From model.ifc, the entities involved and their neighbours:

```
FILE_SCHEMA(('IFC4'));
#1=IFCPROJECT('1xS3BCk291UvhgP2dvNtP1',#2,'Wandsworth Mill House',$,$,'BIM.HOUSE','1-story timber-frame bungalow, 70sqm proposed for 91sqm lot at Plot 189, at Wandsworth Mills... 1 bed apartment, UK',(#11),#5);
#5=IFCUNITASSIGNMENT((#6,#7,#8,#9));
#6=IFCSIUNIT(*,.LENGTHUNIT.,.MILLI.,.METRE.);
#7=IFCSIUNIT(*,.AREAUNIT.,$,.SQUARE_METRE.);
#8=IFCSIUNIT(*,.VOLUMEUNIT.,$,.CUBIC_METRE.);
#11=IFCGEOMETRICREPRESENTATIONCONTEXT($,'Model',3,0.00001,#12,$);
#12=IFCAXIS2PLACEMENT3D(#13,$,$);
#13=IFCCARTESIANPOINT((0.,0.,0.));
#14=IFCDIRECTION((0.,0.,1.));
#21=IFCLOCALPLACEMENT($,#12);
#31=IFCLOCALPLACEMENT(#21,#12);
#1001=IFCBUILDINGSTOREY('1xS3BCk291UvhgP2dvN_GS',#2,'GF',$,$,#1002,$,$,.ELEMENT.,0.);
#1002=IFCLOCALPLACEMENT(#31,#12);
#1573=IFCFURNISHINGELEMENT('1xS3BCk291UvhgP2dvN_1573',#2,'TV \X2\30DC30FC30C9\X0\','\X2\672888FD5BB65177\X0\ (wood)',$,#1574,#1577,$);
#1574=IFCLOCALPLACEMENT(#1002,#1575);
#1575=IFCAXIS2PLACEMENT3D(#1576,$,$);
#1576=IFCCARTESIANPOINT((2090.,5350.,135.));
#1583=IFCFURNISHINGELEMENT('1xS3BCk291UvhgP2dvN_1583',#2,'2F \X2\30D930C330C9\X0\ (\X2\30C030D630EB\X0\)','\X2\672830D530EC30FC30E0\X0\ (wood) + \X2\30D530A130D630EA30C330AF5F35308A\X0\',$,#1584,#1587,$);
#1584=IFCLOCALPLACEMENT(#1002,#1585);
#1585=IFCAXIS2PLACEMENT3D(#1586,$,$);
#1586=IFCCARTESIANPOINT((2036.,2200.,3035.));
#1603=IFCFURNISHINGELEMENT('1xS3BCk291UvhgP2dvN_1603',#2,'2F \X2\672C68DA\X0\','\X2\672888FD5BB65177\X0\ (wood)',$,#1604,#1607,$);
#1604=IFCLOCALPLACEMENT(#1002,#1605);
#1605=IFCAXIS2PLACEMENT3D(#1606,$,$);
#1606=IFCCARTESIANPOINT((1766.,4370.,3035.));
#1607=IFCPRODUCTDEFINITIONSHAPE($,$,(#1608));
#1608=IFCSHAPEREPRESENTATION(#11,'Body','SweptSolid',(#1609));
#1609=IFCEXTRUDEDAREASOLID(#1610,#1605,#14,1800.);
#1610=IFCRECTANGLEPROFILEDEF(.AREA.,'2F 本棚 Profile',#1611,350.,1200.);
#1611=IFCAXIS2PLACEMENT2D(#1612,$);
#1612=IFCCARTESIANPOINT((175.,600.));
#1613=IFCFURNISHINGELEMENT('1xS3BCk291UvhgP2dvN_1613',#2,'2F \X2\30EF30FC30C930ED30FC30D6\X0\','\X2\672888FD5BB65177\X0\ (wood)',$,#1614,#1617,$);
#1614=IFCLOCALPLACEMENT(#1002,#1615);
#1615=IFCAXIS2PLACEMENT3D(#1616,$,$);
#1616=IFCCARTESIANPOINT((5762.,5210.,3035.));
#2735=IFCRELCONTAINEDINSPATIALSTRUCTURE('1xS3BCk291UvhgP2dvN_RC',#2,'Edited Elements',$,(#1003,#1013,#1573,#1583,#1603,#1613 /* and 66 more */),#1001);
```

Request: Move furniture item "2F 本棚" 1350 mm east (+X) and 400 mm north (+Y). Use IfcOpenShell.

```python
import ifcopenshell
import ifcopenshell.api.geometry
import ifcopenshell.util.placement

model = ifcopenshell.open("model.ifc")

item = model.by_guid("1xS3BCk291UvhgP2dvN_1603")
matrix = ifcopenshell.util.placement.get_local_placement(item.ObjectPlacement)
matrix[0, 3] += 1350.0
matrix[1, 3] += 400.0
ifcopenshell.api.geometry.edit_object_placement(model, product=item, matrix=matrix, is_si=False)

print(ifcopenshell.util.placement.get_local_placement(item.ObjectPlacement).round(3) + 0.0)

model.write("model_rev.ifc")
```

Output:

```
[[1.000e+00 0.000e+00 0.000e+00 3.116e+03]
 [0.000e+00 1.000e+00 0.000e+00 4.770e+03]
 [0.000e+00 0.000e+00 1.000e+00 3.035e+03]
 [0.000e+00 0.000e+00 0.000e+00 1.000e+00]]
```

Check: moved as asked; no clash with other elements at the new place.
